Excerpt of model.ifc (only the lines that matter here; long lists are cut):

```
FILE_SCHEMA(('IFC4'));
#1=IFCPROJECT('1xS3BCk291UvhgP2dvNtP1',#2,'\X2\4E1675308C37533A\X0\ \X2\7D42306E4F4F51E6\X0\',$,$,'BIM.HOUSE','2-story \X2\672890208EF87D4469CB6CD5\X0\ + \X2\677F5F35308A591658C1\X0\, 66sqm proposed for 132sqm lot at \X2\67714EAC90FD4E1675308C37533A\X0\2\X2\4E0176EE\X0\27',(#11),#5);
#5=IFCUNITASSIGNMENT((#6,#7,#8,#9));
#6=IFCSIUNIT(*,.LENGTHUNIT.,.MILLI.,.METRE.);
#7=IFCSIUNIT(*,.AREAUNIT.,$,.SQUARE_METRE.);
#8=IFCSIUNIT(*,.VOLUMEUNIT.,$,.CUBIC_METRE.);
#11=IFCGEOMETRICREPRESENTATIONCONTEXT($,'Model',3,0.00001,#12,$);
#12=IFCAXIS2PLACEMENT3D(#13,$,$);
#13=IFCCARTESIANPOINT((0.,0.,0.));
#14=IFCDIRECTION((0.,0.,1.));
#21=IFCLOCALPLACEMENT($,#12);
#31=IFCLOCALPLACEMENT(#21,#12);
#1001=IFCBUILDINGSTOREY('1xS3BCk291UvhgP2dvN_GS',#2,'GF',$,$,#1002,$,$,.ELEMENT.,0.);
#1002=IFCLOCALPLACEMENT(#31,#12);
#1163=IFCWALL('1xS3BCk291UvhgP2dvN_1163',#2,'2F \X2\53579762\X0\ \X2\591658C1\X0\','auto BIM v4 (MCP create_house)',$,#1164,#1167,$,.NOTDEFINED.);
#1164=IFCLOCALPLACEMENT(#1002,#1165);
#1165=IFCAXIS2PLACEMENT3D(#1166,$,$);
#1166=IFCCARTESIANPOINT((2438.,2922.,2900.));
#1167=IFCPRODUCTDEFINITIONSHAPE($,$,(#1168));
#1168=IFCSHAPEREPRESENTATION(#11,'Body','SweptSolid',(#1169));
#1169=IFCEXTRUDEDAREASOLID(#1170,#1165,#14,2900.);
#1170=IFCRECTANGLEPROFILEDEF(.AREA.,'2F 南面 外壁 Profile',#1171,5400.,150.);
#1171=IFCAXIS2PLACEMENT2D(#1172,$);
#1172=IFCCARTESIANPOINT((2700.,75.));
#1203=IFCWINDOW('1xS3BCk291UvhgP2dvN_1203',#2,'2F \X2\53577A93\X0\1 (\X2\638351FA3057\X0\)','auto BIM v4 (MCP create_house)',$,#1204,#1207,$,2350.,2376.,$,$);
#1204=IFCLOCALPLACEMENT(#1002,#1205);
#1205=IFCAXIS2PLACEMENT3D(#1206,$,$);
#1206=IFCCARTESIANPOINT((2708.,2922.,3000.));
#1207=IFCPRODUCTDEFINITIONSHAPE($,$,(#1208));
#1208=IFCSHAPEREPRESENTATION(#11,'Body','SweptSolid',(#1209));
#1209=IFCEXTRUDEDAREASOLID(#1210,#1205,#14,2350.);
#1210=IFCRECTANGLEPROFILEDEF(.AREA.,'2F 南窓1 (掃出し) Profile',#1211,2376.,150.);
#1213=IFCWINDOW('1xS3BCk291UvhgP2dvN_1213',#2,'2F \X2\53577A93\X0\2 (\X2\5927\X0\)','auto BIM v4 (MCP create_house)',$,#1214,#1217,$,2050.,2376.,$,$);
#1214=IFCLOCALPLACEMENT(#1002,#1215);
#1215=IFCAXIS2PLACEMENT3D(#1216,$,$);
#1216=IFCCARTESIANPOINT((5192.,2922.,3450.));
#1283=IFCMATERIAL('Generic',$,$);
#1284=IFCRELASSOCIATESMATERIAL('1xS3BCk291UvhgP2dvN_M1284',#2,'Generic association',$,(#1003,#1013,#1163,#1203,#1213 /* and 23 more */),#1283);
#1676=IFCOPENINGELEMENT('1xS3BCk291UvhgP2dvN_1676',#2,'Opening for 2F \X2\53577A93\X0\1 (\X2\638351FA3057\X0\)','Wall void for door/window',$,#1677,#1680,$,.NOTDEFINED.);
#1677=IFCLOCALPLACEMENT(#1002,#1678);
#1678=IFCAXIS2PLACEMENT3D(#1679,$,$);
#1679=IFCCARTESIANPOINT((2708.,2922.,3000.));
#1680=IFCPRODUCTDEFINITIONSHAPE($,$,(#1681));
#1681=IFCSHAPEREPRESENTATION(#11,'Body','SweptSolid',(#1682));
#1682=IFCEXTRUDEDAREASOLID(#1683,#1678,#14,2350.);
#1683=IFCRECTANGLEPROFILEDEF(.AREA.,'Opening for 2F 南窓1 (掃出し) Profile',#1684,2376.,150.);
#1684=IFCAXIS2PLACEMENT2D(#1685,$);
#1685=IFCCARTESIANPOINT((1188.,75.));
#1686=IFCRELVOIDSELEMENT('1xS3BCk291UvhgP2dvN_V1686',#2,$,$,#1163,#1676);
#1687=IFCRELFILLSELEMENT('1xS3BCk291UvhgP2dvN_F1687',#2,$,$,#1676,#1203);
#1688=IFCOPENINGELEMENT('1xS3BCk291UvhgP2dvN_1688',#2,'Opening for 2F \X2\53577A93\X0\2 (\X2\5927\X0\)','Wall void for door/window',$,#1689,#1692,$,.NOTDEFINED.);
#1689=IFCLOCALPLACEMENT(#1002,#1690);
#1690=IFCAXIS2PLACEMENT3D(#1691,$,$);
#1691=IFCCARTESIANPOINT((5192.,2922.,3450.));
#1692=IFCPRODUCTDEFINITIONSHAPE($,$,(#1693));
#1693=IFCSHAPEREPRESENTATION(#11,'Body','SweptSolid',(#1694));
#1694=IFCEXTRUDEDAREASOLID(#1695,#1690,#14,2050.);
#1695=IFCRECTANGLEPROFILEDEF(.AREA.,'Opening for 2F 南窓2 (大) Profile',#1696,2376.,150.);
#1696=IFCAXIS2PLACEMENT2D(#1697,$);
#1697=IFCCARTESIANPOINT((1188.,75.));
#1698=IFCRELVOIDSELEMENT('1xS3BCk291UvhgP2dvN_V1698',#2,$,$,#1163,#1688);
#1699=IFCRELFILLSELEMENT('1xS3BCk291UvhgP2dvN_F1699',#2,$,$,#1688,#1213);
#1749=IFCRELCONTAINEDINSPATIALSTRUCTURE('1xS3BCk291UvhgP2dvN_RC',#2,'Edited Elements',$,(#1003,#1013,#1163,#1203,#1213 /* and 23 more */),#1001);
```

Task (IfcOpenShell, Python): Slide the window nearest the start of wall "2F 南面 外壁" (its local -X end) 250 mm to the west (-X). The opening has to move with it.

```python
import ifcopenshell
import ifcopenshell.api.geometry
import ifcopenshell.util.placement

model = ifcopenshell.open("model.ifc")

window = model.by_id(1203)
opening = window.FillsVoids[0].RelatingOpeningElement
wall = opening.VoidsElements[0].RelatingBuildingElement

wall_matrix = ifcopenshell.util.placement.get_local_placement(wall.ObjectPlacement)
shift = wall_matrix[:3, 0] * -250.0
before = ifcopenshell.util.placement.get_local_placement(window.ObjectPlacement)[:3, 3].copy()

# The window is not placed relative to its opening, so move both.
for product in (opening, window):
    matrix = ifcopenshell.util.placement.get_local_placement(product.ObjectPlacement)
    matrix[:3, 3] += shift
    ifcopenshell.api.geometry.edit_object_placement(model, product=product, matrix=matrix, is_si=False)

after = ifcopenshell.util.placement.get_local_placement(window.ObjectPlacement)[:3, 3]
print("window moved by", (after - before).round(3) + 0.0)

model.write("model_rev.ifc")
```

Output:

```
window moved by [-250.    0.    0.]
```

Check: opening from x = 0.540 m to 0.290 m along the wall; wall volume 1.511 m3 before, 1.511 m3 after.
